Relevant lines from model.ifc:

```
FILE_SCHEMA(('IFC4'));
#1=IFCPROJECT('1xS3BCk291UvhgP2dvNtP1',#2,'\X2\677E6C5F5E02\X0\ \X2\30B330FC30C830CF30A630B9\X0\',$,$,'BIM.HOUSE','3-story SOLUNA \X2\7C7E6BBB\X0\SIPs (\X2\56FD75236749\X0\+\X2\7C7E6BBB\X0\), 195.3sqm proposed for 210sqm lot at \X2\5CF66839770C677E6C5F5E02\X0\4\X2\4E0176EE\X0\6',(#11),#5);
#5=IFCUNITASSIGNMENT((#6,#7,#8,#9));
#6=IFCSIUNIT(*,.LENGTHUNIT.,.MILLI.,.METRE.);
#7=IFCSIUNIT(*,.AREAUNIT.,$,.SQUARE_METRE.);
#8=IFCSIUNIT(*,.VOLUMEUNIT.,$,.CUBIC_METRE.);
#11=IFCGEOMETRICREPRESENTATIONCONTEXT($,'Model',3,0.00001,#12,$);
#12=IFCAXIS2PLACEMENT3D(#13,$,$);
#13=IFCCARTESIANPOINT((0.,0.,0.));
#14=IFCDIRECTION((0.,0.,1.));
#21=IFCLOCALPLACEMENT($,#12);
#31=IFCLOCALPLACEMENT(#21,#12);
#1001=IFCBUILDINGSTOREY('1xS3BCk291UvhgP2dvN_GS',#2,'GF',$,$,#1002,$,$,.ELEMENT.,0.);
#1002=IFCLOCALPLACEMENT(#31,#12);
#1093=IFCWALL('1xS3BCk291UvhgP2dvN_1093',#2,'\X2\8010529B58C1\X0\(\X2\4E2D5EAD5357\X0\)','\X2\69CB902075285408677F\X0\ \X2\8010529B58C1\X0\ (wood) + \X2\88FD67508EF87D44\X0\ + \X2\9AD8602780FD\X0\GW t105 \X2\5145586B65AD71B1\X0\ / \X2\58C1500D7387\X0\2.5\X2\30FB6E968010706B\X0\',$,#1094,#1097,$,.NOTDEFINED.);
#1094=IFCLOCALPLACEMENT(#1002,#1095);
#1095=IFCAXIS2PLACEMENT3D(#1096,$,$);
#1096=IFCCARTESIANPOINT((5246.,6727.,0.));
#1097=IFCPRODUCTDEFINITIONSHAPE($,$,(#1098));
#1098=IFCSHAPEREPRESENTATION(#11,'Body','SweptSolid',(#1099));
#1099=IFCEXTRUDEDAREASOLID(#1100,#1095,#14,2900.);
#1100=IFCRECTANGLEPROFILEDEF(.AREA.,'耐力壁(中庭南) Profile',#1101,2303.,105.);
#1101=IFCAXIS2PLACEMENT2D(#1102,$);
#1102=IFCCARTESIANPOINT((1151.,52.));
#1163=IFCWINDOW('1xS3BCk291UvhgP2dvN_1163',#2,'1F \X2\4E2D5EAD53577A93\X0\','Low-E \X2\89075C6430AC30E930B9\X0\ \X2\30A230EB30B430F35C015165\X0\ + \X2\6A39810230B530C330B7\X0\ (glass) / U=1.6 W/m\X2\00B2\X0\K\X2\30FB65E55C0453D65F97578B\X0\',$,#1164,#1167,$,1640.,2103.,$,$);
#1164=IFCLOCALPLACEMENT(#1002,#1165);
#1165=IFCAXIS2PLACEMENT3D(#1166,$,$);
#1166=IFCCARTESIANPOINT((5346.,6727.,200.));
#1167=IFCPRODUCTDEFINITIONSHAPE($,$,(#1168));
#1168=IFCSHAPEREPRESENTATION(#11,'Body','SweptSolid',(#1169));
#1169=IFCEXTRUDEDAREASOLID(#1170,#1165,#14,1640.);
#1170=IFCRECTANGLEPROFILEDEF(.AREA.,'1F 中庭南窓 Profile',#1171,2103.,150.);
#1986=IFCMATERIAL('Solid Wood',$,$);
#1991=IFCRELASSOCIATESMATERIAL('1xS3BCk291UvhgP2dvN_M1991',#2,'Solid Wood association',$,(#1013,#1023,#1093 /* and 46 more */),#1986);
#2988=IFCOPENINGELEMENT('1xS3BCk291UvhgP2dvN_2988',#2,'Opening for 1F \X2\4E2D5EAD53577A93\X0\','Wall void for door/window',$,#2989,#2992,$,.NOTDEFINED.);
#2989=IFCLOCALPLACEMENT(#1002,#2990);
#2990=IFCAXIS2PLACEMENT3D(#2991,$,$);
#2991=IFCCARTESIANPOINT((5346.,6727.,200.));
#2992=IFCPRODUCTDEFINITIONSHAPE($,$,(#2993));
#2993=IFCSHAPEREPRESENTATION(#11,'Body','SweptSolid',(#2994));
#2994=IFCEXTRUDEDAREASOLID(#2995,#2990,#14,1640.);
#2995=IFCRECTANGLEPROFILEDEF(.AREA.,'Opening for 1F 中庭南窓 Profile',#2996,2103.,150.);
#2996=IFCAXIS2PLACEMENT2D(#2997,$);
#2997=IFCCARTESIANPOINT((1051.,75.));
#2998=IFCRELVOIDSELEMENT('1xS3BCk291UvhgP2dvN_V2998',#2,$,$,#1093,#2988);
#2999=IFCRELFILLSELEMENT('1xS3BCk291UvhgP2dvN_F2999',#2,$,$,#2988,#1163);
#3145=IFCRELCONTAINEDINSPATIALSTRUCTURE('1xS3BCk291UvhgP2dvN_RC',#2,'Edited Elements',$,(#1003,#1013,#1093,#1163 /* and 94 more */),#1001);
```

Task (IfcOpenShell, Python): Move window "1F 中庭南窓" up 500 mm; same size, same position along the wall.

```python
import numpy as np
import ifcopenshell
import ifcopenshell.api.geometry
import ifcopenshell.util.placement
import ifcopenshell.util.unit

model = ifcopenshell.open("model.ifc")
unit_scale = ifcopenshell.util.unit.calculate_unit_scale(model)

window = model.by_guid("1xS3BCk291UvhgP2dvN_1163")
opening = window.FillsVoids[0].RelatingOpeningElement
dz = 500.0

shift = np.array([0.0, 0.0, dz])
# The window is not placed relative to its opening, so move both.
for product in (opening, window):
    matrix = ifcopenshell.util.placement.get_local_placement(product.ObjectPlacement)
    matrix[:3, 3] += shift
    ifcopenshell.api.geometry.edit_object_placement(model, product=product, matrix=matrix, is_si=False)

print(f"moved by {dz * unit_scale:+.3f} m")

model.write("model_edited.ifc")
```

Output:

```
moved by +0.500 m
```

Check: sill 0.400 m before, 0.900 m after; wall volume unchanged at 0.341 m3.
